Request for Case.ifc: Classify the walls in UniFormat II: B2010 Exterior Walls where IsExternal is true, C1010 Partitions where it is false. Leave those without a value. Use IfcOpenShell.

First a look at what the model holds.

```python
import ifcopenshell
import ifcopenshell.util.element

model = ifcopenshell.open("Case.ifc")
print(model.schema)
print("classifications:", [c.Name for c in model.by_type("IfcClassification")])
values = [ifcopenshell.util.element.get_pset(e, "Pset_WallCommon", "IsExternal") for e in model.by_type("IfcWall")]
for value in (True, False, None):
    print("IsExternal", value, values.count(value))
```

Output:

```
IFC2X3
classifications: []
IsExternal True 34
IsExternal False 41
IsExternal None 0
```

```python
import ifcopenshell
import ifcopenshell.api.classification
import ifcopenshell.util.element

model = ifcopenshell.open("Case.ifc")

# IFC2X3 requires Source and Edition and has no link from the project to the system.
system = model.create_entity("IfcClassification", Source="ASTM", Edition="E1557", Name="UniFormat II")

walls = model.by_type("IfcWall")
external = {e: ifcopenshell.util.element.get_pset(e, "Pset_WallCommon", "IsExternal") for e in walls}
for flag, code, name in ((True, "B2010", "Exterior Walls"), (False, "C1010", "Partitions")):
    products = [e for e in walls if external[e] is flag]
    ifcopenshell.api.classification.add_reference(
        model, products=products, classification=system, identification=code, name=name
    )
    print(code, len(products))

model.write("Case_updated.ifc")
```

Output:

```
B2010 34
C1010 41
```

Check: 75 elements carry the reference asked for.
